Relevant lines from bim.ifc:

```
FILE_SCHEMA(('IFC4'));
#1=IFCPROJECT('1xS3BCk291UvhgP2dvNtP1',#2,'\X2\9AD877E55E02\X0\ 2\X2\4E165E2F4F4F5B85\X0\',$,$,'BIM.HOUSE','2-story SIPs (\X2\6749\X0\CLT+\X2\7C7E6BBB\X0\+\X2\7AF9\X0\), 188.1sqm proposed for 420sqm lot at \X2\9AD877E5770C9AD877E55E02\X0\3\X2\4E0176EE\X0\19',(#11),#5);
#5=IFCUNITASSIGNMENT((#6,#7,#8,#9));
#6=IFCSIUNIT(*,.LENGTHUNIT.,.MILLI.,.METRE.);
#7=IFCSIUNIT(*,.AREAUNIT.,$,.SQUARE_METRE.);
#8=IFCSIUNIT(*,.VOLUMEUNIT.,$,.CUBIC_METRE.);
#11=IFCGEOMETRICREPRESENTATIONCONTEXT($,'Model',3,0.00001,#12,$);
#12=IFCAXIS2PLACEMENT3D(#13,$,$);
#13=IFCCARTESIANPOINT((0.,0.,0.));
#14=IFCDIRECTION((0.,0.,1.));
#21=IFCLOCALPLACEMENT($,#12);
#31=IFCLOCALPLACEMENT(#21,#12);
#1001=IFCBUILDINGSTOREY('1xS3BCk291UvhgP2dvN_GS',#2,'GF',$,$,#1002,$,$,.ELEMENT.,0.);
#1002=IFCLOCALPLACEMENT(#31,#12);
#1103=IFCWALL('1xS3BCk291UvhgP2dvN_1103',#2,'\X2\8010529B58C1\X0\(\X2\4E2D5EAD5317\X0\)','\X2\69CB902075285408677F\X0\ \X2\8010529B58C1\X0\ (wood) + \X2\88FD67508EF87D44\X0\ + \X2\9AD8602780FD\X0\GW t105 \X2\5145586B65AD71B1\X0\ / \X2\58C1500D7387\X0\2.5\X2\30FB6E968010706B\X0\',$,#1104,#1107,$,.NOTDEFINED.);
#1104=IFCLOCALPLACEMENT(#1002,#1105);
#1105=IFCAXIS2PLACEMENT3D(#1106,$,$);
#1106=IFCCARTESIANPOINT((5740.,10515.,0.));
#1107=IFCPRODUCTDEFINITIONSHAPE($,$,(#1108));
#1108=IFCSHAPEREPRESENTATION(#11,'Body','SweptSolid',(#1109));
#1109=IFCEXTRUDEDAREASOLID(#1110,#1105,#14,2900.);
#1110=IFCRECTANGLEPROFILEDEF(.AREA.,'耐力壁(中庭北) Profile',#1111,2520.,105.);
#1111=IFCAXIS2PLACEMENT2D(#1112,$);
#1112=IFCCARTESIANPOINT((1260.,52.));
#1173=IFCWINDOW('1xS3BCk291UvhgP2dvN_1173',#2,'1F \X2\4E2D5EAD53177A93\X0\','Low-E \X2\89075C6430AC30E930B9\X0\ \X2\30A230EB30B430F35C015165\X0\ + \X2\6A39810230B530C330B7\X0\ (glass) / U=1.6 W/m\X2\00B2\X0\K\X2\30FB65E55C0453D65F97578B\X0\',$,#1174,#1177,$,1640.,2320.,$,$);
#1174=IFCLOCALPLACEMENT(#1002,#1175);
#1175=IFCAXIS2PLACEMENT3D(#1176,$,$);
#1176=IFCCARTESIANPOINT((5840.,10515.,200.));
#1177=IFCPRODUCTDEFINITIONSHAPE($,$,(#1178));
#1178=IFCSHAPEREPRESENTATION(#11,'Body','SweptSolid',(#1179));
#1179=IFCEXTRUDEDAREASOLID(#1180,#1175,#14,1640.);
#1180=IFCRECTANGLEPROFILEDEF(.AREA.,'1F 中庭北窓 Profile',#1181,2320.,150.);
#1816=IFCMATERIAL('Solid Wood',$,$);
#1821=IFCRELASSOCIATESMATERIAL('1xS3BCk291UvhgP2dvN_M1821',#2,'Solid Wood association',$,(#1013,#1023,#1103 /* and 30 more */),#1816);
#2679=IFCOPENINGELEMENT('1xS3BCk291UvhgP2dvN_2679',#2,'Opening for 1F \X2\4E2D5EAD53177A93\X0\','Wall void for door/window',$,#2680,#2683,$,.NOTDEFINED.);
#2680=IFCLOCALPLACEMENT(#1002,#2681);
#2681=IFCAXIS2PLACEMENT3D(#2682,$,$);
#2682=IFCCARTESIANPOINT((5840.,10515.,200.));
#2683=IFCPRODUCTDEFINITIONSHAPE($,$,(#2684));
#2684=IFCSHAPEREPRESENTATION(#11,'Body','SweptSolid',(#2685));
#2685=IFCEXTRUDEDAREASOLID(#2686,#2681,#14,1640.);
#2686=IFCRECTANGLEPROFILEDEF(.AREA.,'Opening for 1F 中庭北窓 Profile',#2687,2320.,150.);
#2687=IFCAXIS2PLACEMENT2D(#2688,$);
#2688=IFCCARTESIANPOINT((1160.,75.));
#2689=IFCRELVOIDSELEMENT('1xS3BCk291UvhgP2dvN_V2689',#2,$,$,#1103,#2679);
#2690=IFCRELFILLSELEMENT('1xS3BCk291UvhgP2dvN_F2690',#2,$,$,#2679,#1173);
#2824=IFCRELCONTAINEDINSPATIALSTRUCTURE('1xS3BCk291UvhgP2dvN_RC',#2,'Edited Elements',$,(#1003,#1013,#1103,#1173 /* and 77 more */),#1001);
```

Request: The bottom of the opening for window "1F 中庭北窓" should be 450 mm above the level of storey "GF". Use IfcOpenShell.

```python
import numpy as np
import ifcopenshell
import ifcopenshell.api.geometry
import ifcopenshell.geom
import ifcopenshell.util.element
import ifcopenshell.util.placement
import ifcopenshell.util.shape
import ifcopenshell.util.unit

model = ifcopenshell.open("bim.ifc")
unit_scale = ifcopenshell.util.unit.calculate_unit_scale(model)

window = model.by_id(1173)
opening = window.FillsVoids[0].RelatingOpeningElement
storey = ifcopenshell.util.element.get_container(window, ifc_class="IfcBuildingStorey")
level = ifcopenshell.util.placement.get_local_placement(storey.ObjectPlacement)[2, 3]

# The opening's origin need not be at the sill, so measure its lowest point.
shape = ifcopenshell.geom.create_shape(ifcopenshell.geom.settings(), opening)
bottom = ifcopenshell.util.shape.get_shape_bottom_elevation(shape, shape.geometry) / unit_scale
dz = level + 0.45 / unit_scale - bottom

shift = np.array([0.0, 0.0, dz])
# The window is not placed relative to its opening, so move both.
for product in (opening, window):
    matrix = ifcopenshell.util.placement.get_local_placement(product.ObjectPlacement)
    matrix[:3, 3] += shift
    ifcopenshell.api.geometry.edit_object_placement(model, product=product, matrix=matrix, is_si=False)

print(f"moved by {dz * unit_scale:+.3f} m")

model.write("bim-out.ifc")
```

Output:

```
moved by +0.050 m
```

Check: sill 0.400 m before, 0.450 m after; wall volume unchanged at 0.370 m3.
